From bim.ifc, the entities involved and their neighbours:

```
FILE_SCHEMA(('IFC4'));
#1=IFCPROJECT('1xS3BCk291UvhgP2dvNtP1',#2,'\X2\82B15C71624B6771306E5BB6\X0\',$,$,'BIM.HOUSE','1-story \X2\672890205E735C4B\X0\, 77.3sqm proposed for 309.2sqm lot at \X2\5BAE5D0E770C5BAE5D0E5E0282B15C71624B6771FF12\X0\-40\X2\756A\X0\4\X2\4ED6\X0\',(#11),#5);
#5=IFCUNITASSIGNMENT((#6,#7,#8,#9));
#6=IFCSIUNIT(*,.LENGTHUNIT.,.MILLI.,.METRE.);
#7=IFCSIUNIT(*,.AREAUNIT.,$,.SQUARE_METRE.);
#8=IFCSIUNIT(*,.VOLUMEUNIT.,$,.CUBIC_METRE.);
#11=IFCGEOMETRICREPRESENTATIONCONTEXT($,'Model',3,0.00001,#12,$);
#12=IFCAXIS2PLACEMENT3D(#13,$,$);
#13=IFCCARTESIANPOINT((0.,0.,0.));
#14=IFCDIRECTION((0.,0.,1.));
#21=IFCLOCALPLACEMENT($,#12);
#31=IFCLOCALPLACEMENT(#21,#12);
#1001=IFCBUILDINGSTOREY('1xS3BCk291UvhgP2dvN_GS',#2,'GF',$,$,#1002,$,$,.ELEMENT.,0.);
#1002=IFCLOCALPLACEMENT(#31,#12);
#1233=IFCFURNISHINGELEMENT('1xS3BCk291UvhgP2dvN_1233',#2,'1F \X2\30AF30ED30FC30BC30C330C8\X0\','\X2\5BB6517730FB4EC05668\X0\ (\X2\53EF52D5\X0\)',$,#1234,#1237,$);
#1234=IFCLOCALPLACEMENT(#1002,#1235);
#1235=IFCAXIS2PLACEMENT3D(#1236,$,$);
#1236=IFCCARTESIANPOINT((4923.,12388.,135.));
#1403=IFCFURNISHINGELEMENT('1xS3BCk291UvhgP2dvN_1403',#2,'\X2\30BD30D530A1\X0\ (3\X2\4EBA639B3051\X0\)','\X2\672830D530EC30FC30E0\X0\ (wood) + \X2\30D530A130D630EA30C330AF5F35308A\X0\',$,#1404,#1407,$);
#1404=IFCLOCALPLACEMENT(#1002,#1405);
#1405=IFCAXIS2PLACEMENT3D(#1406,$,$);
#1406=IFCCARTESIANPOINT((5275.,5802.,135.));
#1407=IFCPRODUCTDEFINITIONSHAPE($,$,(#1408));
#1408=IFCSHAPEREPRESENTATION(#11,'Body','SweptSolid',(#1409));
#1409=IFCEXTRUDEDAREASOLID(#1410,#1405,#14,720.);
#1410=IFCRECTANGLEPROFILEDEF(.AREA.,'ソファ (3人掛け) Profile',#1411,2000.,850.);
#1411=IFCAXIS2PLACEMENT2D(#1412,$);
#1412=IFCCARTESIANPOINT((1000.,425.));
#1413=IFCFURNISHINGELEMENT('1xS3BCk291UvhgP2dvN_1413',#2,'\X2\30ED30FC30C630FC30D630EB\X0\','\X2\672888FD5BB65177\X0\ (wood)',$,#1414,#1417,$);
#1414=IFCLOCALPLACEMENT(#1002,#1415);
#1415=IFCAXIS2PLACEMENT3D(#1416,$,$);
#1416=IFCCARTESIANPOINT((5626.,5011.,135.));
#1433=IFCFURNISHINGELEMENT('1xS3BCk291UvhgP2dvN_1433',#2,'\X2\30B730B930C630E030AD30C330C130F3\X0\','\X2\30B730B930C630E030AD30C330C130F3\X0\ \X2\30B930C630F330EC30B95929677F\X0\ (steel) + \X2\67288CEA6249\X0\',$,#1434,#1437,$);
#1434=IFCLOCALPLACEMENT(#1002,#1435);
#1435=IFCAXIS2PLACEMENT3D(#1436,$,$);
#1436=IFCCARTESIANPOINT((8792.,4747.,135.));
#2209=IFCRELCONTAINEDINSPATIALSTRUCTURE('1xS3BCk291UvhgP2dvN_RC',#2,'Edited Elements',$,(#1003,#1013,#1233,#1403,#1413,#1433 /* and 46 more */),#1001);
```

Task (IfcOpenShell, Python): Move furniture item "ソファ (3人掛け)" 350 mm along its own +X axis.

```python
import ifcopenshell
import ifcopenshell.api.geometry
import ifcopenshell.util.placement
import ifcopenshell.util.unit

model = ifcopenshell.open("bim.ifc")
unit_scale = ifcopenshell.util.unit.calculate_unit_scale(model)

item = model.by_guid("1xS3BCk291UvhgP2dvN_1403")
matrix = ifcopenshell.util.placement.get_local_placement(item.ObjectPlacement)
matrix[:3, 3] += matrix[:3, 0] * 0.35 / unit_scale
ifcopenshell.api.geometry.edit_object_placement(model, product=item, matrix=matrix, is_si=False)

print(ifcopenshell.util.placement.get_local_placement(item.ObjectPlacement).round(3) + 0.0)

model.write("bim_updated.ifc")
```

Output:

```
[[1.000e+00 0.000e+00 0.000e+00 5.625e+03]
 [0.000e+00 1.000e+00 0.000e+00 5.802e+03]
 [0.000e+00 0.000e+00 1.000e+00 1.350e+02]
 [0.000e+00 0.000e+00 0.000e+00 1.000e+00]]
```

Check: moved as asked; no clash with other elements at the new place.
